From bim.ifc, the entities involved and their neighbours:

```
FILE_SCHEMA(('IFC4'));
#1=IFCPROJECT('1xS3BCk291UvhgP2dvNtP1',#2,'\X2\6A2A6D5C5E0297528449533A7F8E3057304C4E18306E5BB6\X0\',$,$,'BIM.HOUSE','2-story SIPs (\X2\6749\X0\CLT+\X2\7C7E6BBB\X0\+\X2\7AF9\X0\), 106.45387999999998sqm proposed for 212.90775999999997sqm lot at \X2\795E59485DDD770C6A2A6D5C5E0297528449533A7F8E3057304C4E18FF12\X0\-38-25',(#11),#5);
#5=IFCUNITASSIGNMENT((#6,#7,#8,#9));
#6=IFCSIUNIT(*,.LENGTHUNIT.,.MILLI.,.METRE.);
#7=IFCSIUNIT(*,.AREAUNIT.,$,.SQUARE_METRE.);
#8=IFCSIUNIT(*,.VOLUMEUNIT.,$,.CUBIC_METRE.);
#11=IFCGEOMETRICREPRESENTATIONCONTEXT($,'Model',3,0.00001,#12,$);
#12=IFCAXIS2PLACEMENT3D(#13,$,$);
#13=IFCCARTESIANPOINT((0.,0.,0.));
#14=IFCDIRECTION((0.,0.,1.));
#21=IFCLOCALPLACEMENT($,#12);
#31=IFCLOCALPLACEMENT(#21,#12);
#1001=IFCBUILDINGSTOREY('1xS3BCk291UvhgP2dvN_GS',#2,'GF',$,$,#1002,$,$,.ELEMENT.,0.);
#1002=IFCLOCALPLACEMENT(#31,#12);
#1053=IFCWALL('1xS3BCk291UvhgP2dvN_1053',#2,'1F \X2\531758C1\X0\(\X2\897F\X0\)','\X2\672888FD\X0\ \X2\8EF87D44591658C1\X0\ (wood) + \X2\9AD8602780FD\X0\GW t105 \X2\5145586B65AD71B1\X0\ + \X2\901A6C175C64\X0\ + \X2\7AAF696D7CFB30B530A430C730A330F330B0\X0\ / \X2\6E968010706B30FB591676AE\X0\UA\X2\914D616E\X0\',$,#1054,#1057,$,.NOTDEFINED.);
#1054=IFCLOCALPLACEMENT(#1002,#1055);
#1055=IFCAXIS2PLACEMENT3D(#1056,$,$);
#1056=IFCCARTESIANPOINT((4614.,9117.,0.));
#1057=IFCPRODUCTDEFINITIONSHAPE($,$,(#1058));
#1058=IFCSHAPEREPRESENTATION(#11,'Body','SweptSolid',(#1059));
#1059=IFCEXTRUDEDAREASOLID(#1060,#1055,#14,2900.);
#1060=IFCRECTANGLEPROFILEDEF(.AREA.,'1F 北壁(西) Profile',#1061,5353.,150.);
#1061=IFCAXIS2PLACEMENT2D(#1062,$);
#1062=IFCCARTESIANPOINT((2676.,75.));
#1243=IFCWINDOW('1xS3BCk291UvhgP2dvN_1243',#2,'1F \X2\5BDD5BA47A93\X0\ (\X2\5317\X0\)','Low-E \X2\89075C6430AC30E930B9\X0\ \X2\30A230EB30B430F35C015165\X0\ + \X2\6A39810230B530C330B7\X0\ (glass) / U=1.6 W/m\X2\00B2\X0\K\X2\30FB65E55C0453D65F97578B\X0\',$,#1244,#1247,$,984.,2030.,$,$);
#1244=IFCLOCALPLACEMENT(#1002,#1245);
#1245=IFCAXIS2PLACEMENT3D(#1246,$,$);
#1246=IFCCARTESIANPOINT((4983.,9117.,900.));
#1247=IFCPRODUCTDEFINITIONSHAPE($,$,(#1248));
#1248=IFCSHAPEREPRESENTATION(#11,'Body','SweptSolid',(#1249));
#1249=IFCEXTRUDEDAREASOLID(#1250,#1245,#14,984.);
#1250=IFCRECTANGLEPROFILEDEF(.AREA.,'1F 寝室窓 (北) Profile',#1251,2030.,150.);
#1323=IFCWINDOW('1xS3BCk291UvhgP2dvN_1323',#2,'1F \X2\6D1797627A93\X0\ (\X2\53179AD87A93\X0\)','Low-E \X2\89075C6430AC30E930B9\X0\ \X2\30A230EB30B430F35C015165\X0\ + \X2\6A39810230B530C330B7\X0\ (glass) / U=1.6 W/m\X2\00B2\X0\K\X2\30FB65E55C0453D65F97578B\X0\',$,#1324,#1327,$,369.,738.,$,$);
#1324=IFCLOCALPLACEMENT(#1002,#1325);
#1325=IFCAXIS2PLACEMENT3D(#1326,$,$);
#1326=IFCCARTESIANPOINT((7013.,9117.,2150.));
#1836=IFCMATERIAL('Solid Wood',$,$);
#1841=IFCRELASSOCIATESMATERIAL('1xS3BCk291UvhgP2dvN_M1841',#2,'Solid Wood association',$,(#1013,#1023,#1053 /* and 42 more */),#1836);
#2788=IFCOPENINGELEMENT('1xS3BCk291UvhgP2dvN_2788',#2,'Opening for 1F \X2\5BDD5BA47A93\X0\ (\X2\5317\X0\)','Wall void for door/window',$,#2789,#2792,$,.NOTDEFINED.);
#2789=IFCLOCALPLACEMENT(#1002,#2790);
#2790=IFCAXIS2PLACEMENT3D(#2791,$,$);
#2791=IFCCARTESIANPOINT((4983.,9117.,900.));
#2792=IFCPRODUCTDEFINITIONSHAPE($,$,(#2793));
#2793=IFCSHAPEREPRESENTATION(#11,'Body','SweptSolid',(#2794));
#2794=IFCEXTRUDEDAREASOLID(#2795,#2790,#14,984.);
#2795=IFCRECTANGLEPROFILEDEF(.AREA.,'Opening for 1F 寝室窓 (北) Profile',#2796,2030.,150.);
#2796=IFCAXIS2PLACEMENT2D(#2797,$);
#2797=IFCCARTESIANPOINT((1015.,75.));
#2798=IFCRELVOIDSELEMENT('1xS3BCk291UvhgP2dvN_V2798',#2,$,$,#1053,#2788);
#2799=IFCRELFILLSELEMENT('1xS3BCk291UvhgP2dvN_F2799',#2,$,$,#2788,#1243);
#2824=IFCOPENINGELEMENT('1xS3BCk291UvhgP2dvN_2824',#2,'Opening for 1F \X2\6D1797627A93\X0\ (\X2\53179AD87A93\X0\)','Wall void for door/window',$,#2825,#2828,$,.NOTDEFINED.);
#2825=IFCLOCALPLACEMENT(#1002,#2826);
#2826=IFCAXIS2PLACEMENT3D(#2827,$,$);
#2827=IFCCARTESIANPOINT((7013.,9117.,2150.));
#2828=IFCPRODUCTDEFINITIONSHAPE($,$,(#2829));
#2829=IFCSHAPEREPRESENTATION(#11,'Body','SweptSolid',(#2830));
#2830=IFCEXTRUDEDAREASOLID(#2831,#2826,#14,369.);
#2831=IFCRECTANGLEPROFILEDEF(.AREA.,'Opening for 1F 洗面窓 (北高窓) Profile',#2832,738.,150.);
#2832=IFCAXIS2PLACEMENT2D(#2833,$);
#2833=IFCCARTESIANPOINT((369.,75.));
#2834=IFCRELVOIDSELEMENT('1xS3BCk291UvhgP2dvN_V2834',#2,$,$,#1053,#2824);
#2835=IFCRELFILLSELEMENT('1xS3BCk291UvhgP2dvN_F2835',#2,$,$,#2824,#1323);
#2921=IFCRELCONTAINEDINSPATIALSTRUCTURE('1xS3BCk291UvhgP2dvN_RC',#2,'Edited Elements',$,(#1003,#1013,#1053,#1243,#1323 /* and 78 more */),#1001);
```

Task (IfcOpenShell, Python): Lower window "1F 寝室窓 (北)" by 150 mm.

```python
import numpy as np
import ifcopenshell
import ifcopenshell.api.geometry
import ifcopenshell.util.placement
import ifcopenshell.util.unit

model = ifcopenshell.open("bim.ifc")
unit_scale = ifcopenshell.util.unit.calculate_unit_scale(model)

window = model.by_guid("1xS3BCk291UvhgP2dvN_1243")
opening = window.FillsVoids[0].RelatingOpeningElement
dz = -0.15 / unit_scale

shift = np.array([0.0, 0.0, dz])
# The window is not placed relative to its opening, so move both.
for product in (opening, window):
    matrix = ifcopenshell.util.placement.get_local_placement(product.ObjectPlacement)
    matrix[:3, 3] += shift
    ifcopenshell.api.geometry.edit_object_placement(model, product=product, matrix=matrix, is_si=False)

print(f"moved by {dz * unit_scale:+.3f} m")

model.write("bim_v2.ifc")
```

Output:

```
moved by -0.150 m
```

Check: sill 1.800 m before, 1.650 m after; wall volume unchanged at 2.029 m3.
